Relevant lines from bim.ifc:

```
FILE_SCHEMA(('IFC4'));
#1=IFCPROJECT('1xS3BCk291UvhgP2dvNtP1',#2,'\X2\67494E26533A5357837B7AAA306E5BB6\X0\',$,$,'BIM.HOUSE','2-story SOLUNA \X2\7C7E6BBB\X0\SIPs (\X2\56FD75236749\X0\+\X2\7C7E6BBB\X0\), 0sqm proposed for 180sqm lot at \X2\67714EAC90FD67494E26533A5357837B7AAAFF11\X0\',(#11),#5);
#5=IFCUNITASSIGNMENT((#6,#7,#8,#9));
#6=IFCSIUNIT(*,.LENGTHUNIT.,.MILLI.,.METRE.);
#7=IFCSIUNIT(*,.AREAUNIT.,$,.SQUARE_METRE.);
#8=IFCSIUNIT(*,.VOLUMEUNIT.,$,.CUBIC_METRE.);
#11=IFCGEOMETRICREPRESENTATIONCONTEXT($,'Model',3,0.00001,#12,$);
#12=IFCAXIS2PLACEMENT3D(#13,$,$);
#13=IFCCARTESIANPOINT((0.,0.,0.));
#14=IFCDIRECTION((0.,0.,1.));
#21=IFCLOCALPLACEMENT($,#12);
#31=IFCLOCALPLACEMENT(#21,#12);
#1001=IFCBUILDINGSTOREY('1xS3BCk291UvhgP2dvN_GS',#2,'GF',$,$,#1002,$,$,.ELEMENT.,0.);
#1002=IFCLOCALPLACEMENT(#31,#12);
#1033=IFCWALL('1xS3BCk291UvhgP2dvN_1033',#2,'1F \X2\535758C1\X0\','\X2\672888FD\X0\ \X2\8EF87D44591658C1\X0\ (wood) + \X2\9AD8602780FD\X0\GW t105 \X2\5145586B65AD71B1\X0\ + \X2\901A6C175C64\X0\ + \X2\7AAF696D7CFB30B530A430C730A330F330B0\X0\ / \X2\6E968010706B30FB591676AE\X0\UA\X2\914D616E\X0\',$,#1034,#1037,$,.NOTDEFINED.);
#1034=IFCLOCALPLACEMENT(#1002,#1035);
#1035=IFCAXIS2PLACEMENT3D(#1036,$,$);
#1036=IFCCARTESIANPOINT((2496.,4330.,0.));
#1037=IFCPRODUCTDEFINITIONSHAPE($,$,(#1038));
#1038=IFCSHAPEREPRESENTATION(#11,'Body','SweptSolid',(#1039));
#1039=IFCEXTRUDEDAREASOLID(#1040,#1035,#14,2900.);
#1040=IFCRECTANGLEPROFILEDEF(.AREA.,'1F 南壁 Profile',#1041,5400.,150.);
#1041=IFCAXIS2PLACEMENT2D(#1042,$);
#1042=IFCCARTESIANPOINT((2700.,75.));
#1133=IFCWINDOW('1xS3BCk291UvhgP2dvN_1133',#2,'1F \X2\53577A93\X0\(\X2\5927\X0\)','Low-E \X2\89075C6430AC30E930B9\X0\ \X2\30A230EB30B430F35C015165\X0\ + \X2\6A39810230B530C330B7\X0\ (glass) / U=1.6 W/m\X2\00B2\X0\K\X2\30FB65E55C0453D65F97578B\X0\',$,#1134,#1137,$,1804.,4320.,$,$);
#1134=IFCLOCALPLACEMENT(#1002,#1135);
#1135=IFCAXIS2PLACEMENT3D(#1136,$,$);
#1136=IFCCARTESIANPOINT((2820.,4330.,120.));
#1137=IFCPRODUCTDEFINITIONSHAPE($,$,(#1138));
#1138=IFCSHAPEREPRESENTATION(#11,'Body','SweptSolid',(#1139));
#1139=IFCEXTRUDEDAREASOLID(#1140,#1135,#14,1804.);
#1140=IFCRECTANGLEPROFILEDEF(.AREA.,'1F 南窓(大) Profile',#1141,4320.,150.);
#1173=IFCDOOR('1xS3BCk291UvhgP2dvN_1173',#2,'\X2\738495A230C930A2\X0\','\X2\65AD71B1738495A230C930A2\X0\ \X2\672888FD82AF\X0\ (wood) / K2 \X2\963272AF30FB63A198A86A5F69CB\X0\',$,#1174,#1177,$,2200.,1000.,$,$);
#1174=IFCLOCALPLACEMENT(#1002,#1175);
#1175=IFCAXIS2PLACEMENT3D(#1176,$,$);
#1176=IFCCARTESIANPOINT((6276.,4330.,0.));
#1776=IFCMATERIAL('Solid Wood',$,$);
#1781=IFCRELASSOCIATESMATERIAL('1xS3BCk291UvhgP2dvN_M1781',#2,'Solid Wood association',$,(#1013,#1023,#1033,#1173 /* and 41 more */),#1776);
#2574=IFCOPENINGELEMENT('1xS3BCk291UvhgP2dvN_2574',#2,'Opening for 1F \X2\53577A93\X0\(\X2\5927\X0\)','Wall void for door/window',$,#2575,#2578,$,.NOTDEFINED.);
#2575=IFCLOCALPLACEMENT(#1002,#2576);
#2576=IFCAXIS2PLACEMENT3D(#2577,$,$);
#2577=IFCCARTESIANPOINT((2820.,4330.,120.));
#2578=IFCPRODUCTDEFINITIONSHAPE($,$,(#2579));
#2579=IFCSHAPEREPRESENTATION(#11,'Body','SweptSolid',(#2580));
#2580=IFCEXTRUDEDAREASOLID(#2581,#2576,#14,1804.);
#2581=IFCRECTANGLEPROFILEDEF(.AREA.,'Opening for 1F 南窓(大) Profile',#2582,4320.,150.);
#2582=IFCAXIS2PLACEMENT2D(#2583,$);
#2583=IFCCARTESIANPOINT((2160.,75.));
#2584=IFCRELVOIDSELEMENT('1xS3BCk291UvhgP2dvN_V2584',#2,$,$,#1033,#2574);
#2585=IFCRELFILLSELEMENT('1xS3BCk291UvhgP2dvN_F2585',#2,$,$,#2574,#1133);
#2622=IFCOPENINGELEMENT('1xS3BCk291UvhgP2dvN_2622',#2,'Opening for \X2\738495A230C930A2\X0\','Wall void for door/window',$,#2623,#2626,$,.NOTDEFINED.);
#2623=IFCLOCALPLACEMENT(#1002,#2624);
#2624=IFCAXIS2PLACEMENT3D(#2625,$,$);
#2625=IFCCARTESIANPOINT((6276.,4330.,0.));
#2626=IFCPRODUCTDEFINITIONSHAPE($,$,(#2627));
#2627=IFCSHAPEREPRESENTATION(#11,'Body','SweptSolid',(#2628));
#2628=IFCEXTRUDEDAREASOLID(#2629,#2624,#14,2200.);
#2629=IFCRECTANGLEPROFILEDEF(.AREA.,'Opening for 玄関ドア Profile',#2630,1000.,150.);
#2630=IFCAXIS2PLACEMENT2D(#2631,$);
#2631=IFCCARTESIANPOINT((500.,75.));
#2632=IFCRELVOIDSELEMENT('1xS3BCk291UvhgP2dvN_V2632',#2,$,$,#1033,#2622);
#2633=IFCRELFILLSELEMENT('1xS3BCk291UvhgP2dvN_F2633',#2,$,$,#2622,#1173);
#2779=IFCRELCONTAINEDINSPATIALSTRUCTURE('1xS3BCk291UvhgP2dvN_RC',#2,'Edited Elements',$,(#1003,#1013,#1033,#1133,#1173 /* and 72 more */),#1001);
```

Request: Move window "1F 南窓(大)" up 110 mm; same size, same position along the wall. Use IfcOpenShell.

```python
import numpy as np
import ifcopenshell
import ifcopenshell.api.geometry
import ifcopenshell.util.placement
import ifcopenshell.util.unit

model = ifcopenshell.open("bim.ifc")
unit_scale = ifcopenshell.util.unit.calculate_unit_scale(model)

window = model.by_guid("1xS3BCk291UvhgP2dvN_1133")
opening = window.FillsVoids[0].RelatingOpeningElement
dz = 0.11 / unit_scale

shift = np.array([0.0, 0.0, dz])
# The window is not placed relative to its opening, so move both.
for product in (opening, window):
    matrix = ifcopenshell.util.placement.get_local_placement(product.ObjectPlacement)
    matrix[:3, 3] += shift
    ifcopenshell.api.geometry.edit_object_placement(model, product=product, matrix=matrix, is_si=False)

print(f"moved by {dz * unit_scale:+.3f} m")

model.write("bim-out.ifc")
```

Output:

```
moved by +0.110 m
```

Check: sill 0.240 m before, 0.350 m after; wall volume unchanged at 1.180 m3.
